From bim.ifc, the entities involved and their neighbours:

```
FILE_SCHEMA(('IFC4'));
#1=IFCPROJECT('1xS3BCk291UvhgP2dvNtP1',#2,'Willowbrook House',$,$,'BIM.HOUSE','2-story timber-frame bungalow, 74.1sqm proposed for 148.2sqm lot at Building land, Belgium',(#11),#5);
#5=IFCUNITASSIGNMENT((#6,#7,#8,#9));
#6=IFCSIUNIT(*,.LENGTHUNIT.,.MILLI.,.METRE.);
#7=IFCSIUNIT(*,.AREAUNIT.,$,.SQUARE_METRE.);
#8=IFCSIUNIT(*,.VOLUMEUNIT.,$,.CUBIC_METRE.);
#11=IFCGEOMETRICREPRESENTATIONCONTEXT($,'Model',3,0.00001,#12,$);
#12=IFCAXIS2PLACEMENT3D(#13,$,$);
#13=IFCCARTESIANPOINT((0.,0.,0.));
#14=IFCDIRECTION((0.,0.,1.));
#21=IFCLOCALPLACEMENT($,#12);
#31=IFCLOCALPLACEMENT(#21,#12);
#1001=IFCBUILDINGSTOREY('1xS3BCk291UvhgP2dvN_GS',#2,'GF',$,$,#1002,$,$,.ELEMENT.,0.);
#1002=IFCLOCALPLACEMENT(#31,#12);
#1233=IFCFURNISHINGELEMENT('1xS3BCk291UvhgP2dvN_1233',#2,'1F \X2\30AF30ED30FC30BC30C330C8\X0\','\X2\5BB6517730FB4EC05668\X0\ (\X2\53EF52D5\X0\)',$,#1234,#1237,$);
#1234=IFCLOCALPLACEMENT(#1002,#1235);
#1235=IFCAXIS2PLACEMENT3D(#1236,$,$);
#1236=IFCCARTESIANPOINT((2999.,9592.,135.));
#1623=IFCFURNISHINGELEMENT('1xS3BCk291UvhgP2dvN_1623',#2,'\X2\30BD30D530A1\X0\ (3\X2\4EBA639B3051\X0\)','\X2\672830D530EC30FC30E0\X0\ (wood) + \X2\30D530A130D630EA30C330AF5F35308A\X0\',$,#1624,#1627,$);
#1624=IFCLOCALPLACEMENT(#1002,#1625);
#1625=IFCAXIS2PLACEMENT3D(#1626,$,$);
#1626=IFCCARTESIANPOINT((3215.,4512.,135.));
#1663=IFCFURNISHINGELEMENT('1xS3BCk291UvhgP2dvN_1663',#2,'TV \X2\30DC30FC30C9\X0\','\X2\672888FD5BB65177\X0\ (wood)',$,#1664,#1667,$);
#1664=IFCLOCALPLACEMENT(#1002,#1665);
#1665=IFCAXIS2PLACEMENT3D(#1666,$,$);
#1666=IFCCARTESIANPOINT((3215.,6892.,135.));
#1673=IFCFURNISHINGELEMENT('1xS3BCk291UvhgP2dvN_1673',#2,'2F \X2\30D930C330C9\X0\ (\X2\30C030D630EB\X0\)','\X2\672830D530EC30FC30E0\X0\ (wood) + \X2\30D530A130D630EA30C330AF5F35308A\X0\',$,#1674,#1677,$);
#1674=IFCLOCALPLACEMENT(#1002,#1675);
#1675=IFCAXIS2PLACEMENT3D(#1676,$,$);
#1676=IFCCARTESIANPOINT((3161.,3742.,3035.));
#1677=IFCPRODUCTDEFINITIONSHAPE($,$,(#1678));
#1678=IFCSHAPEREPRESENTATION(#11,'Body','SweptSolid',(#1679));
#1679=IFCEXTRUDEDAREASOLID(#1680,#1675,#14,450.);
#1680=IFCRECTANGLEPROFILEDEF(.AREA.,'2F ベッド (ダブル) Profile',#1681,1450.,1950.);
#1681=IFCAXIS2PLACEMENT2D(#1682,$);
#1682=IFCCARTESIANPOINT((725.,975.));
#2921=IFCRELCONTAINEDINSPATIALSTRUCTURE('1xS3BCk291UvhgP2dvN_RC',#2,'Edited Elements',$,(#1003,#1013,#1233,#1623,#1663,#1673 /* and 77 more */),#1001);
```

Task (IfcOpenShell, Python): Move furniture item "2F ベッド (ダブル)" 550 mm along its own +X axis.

```python
import ifcopenshell
import ifcopenshell.api.geometry
import ifcopenshell.util.placement
import ifcopenshell.util.unit

model = ifcopenshell.open("bim.ifc")
unit_scale = ifcopenshell.util.unit.calculate_unit_scale(model)

item = model.by_guid("1xS3BCk291UvhgP2dvN_1673")
matrix = ifcopenshell.util.placement.get_local_placement(item.ObjectPlacement)
matrix[:3, 3] += matrix[:3, 0] * 0.55 / unit_scale
ifcopenshell.api.geometry.edit_object_placement(model, product=item, matrix=matrix, is_si=False)

print(ifcopenshell.util.placement.get_local_placement(item.ObjectPlacement).round(3) + 0.0)

model.write("bim_edited.ifc")
```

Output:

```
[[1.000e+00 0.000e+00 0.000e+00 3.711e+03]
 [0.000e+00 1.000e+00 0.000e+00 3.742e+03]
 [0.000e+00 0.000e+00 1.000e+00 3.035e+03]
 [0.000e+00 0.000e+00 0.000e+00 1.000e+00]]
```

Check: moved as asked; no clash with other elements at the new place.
